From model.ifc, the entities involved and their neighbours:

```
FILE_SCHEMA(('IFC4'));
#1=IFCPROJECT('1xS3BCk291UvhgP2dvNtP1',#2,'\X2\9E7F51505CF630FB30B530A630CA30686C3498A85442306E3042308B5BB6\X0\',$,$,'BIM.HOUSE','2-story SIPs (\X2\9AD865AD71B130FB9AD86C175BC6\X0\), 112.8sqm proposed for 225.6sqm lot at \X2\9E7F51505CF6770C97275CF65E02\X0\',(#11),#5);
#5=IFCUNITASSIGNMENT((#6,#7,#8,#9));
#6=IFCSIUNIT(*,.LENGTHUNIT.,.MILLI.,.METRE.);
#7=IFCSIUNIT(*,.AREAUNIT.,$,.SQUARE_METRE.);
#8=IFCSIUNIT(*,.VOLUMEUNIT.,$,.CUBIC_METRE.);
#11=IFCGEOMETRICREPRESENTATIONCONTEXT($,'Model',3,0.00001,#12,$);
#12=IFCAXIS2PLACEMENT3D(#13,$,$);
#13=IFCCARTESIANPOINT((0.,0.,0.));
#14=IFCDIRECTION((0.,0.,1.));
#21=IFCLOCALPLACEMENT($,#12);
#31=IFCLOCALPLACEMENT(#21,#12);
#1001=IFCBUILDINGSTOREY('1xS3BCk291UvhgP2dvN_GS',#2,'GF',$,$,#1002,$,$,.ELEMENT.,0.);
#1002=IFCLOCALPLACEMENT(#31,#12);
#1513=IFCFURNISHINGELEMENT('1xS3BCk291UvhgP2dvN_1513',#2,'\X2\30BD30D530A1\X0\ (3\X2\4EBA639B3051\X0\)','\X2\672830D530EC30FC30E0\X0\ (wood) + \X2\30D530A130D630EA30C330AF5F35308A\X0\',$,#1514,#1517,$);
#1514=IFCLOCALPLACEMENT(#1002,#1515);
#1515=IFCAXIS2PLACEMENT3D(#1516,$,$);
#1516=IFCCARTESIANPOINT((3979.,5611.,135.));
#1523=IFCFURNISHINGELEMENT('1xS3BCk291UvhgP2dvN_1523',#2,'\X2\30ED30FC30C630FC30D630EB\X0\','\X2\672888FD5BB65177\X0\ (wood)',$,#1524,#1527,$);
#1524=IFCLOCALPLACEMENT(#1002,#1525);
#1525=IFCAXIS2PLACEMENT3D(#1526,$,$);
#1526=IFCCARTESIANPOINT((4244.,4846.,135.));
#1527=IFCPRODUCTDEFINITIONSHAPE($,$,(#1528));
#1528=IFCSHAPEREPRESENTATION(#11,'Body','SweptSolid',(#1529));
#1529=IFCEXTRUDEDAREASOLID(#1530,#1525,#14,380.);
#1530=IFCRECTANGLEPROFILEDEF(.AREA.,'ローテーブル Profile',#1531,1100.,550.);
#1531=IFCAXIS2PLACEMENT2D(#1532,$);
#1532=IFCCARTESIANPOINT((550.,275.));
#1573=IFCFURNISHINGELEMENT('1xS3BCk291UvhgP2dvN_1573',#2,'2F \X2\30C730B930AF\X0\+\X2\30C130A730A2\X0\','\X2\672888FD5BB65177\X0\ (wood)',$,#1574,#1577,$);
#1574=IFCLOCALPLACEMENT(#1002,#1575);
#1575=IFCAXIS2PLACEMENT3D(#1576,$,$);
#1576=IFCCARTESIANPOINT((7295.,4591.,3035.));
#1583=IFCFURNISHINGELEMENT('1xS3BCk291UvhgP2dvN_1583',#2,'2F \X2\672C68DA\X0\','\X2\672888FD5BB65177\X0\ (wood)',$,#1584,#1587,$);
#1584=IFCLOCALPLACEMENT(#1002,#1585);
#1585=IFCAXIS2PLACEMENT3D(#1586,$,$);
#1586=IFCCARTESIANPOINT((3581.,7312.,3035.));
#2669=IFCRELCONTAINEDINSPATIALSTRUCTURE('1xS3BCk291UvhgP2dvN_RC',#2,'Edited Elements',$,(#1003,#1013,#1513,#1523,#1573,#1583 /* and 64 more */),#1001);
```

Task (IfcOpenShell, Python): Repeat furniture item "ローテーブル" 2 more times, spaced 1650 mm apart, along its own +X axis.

```python
import ifcopenshell
import ifcopenshell.api.geometry
import ifcopenshell.api.root
import ifcopenshell.util.element
import ifcopenshell.util.placement

model = ifcopenshell.open("model.ifc")


def reuse_history(source, copy):
    """copy_class also copies each property set's owner history, people and application; keep the originals."""
    for rel in copy.IsDefinedBy:
        if rel.is_a("IfcRelDefinesByProperties") and (history := rel.RelatingPropertyDefinition.OwnerHistory):
            rel.RelatingPropertyDefinition.OwnerHistory = source.OwnerHistory
            ifcopenshell.util.element.remove_deep2(model, history)


source = model.by_guid("1xS3BCk291UvhgP2dvN_1523")
base = ifcopenshell.util.placement.get_local_placement(source.ObjectPlacement)
step = base[:3, 0] * 1650.0

for i in range(1, 3):
    copy = ifcopenshell.api.root.copy_class(model, product=source)
    copy.Representation = ifcopenshell.util.element.copy_deep(
        model, source.Representation, exclude=["IfcGeometricRepresentationContext", "IfcRepresentationMap"]
    )
    reuse_history(source, copy)
    matrix = base.copy()
    matrix[:3, 3] += i * step
    print("added at", matrix[:3, 3].round(3) + 0.0)
    ifcopenshell.api.geometry.edit_object_placement(model, product=copy, matrix=matrix, is_si=False)

model.write("model_updated.ifc")
```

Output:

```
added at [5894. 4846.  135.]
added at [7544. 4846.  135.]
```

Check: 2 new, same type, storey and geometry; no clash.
